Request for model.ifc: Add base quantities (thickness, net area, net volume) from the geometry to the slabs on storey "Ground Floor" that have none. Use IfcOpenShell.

First a look at what the model holds.

```python
import ifcopenshell
import ifcopenshell.util.element
import ifcopenshell.util.unit

model = ifcopenshell.open("model.ifc")
print(model.schema)
for unit_type in ("LENGTHUNIT", "AREAUNIT", "VOLUMEUNIT"):
    print(unit_type, ifcopenshell.util.unit.calculate_unit_scale(model, unit_type))
storey = next(s for s in model.by_type("IfcBuildingStorey") if s.Name == "Ground Floor")
slabs = [e for e in ifcopenshell.util.element.get_decomposition(storey) if e.is_a("IfcSlab")]
for e in sorted(slabs, key=lambda e: e.id()):
    print(e.id(), e.is_a(), e.Name, list(ifcopenshell.util.element.get_psets(e, qtos_only=True)), sep=" | ")
```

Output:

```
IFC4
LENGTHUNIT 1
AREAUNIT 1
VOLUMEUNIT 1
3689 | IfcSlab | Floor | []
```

```python
import ifcopenshell
import ifcopenshell.api.pset
import ifcopenshell.geom
import ifcopenshell.util.element
import ifcopenshell.util.shape
import ifcopenshell.util.unit

model = ifcopenshell.open("model.ifc")
unit_scale = ifcopenshell.util.unit.calculate_unit_scale(model)
area_scale = ifcopenshell.util.unit.calculate_unit_scale(model, "AREAUNIT")
volume_scale = ifcopenshell.util.unit.calculate_unit_scale(model, "VOLUMEUNIT")
settings = ifcopenshell.geom.settings()

storey = next(s for s in model.by_type("IfcBuildingStorey") if s.Name == "Ground Floor")
slabs = [e for e in ifcopenshell.util.element.get_decomposition(storey) if e.is_a("IfcSlab")]

for e in sorted(slabs, key=lambda e: e.id()):
    if ifcopenshell.util.element.get_psets(e, qtos_only=True, should_inherit=False):
        continue
    # Geometry comes back in metres, in the element's own axes.
    shape = ifcopenshell.geom.create_shape(settings, e)
    values = {
        "Width": ifcopenshell.util.shape.get_z(shape.geometry) / unit_scale,
        "NetArea": ifcopenshell.util.shape.get_footprint_area(shape.geometry) / area_scale,
        "NetVolume": ifcopenshell.util.shape.get_volume(shape.geometry) / volume_scale,
    }
    qto = ifcopenshell.api.pset.add_qto(model, product=e, name="Qto_SlabBaseQuantities")
    ifcopenshell.api.pset.edit_qto(model, qto=qto, properties=values)
    print(e.id(), {k: round(v, 3) for k, v in values.items()})

model.write("model_edited.ifc")
```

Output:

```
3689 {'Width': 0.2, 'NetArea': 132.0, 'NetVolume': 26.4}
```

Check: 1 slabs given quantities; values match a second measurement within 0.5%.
